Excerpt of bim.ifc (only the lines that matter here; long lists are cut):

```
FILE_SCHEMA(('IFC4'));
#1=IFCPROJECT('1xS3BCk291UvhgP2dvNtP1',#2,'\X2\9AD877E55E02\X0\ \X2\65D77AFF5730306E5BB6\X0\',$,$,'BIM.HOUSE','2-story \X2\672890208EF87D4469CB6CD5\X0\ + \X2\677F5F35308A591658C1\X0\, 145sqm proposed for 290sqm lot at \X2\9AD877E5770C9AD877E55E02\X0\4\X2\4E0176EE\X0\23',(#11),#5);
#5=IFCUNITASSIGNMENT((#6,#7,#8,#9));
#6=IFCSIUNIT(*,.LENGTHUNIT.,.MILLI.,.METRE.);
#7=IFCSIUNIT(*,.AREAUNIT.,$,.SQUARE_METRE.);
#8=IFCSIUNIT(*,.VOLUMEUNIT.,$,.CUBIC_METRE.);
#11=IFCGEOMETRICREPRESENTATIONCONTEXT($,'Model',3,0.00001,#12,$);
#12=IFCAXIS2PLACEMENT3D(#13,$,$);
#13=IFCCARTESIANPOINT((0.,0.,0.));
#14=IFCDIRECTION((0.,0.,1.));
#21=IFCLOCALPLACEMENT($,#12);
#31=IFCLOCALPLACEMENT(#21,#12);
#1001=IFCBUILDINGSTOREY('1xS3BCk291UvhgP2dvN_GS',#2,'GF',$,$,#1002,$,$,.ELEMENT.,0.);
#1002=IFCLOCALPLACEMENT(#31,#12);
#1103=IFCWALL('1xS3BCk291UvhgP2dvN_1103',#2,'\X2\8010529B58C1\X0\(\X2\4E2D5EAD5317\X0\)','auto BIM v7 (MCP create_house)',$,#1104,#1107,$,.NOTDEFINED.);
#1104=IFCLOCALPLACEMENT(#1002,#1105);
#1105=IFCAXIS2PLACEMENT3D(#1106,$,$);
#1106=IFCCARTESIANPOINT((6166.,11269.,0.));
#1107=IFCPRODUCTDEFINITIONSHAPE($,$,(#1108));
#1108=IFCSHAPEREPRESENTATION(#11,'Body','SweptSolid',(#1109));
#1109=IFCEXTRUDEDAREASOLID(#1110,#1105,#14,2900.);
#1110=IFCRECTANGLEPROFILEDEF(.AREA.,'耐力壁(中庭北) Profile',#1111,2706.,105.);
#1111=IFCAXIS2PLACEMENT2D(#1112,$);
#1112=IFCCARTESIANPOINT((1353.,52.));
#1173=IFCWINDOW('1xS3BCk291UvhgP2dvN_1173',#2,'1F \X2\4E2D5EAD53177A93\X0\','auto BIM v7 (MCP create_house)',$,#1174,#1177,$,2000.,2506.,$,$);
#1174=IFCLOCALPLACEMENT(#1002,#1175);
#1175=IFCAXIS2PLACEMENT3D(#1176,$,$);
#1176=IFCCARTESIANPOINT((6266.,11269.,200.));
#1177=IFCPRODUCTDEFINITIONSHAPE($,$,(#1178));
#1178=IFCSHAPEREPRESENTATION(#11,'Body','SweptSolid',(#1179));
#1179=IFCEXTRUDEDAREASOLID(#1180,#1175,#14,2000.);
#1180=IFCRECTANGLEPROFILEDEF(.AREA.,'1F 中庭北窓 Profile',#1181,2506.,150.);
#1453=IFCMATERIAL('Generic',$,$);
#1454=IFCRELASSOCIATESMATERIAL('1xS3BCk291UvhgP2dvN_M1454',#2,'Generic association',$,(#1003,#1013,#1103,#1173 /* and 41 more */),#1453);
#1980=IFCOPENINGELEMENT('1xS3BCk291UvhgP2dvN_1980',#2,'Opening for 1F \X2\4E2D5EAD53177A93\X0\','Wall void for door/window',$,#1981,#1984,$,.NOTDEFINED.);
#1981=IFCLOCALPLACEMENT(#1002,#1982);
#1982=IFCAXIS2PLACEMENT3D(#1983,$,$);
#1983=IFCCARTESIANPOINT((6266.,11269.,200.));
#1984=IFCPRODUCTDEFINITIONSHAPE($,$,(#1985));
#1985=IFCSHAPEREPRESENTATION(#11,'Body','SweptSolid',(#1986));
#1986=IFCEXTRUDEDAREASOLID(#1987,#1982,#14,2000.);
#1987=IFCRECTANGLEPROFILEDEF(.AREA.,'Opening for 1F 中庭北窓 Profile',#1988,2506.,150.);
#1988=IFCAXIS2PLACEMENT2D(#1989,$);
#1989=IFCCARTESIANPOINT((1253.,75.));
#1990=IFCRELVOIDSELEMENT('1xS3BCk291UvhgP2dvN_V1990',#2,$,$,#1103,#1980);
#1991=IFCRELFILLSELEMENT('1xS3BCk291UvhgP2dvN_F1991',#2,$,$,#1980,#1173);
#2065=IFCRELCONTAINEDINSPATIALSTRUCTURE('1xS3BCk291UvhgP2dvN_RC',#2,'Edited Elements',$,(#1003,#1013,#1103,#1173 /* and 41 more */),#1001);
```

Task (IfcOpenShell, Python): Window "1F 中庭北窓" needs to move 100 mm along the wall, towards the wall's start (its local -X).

```python
import ifcopenshell
import ifcopenshell.api.geometry
import ifcopenshell.util.placement
import ifcopenshell.util.unit

model = ifcopenshell.open("bim.ifc")
unit_scale = ifcopenshell.util.unit.calculate_unit_scale(model)

window = model.by_guid("1xS3BCk291UvhgP2dvN_1173")
opening = window.FillsVoids[0].RelatingOpeningElement
wall = opening.VoidsElements[0].RelatingBuildingElement

wall_matrix = ifcopenshell.util.placement.get_local_placement(wall.ObjectPlacement)
shift = wall_matrix[:3, 0] * -0.1 / unit_scale
before = ifcopenshell.util.placement.get_local_placement(window.ObjectPlacement)[:3, 3].copy()

# The window is not placed relative to its opening, so move both.
for product in (opening, window):
    matrix = ifcopenshell.util.placement.get_local_placement(product.ObjectPlacement)
    matrix[:3, 3] += shift
    ifcopenshell.api.geometry.edit_object_placement(model, product=product, matrix=matrix, is_si=False)

after = ifcopenshell.util.placement.get_local_placement(window.ObjectPlacement)[:3, 3]
print("window moved by", (after - before).round(3) + 0.0)

model.write("bim_edited.ifc")
```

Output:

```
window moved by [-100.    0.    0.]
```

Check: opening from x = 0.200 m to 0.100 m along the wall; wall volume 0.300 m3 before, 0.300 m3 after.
